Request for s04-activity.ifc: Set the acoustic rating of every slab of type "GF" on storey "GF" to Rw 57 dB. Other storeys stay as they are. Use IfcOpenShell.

First a look at what the model holds.

```python
import ifcopenshell
import ifcopenshell.util.element

model = ifcopenshell.open("s04-activity.ifc")
print(model.schema)
storey = next(s for s in model.by_type("IfcBuildingStorey") if s.Name == "GF")
slabs = [e for e in ifcopenshell.util.element.get_decomposition(storey) if e.is_a("IfcSlab")]
seen = {}
for e in slabs:
    element_type = ifcopenshell.util.element.get_type(e)
    key = (element_type.Name if element_type != e and element_type else None, ifcopenshell.util.element.get_pset(e, "Pset_SlabCommon", "AcousticRating"))
    seen[key] = seen.get(key, 0) + 1
for (name, value), count in sorted(seen.items(), key=str):
    print(count, "x", name, "|", value)
```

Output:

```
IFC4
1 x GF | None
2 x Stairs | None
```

```python
import ifcopenshell
import ifcopenshell.api.pset
import ifcopenshell.util.element

model = ifcopenshell.open("s04-activity.ifc")

storey = next(s for s in model.by_type("IfcBuildingStorey") if s.Name == "GF")
slabs = [e for e in ifcopenshell.util.element.get_decomposition(storey) if e.is_a("IfcSlab")]

count = 0
for e in slabs:
    element_type = ifcopenshell.util.element.get_type(e)
    if element_type in (None, e) or element_type.Name != "GF":
        continue
    # add_pset returns the element's existing set when there is one.
    pset = ifcopenshell.api.pset.add_pset(model, product=e, name="Pset_SlabCommon")
    ifcopenshell.api.pset.edit_pset(model, pset=pset, properties={"AcousticRating": "Rw 57 dB"})
    count += 1

print(count, "slabs updated")

model.write("s04-activity_updated.ifc")
```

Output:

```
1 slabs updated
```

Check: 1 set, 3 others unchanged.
